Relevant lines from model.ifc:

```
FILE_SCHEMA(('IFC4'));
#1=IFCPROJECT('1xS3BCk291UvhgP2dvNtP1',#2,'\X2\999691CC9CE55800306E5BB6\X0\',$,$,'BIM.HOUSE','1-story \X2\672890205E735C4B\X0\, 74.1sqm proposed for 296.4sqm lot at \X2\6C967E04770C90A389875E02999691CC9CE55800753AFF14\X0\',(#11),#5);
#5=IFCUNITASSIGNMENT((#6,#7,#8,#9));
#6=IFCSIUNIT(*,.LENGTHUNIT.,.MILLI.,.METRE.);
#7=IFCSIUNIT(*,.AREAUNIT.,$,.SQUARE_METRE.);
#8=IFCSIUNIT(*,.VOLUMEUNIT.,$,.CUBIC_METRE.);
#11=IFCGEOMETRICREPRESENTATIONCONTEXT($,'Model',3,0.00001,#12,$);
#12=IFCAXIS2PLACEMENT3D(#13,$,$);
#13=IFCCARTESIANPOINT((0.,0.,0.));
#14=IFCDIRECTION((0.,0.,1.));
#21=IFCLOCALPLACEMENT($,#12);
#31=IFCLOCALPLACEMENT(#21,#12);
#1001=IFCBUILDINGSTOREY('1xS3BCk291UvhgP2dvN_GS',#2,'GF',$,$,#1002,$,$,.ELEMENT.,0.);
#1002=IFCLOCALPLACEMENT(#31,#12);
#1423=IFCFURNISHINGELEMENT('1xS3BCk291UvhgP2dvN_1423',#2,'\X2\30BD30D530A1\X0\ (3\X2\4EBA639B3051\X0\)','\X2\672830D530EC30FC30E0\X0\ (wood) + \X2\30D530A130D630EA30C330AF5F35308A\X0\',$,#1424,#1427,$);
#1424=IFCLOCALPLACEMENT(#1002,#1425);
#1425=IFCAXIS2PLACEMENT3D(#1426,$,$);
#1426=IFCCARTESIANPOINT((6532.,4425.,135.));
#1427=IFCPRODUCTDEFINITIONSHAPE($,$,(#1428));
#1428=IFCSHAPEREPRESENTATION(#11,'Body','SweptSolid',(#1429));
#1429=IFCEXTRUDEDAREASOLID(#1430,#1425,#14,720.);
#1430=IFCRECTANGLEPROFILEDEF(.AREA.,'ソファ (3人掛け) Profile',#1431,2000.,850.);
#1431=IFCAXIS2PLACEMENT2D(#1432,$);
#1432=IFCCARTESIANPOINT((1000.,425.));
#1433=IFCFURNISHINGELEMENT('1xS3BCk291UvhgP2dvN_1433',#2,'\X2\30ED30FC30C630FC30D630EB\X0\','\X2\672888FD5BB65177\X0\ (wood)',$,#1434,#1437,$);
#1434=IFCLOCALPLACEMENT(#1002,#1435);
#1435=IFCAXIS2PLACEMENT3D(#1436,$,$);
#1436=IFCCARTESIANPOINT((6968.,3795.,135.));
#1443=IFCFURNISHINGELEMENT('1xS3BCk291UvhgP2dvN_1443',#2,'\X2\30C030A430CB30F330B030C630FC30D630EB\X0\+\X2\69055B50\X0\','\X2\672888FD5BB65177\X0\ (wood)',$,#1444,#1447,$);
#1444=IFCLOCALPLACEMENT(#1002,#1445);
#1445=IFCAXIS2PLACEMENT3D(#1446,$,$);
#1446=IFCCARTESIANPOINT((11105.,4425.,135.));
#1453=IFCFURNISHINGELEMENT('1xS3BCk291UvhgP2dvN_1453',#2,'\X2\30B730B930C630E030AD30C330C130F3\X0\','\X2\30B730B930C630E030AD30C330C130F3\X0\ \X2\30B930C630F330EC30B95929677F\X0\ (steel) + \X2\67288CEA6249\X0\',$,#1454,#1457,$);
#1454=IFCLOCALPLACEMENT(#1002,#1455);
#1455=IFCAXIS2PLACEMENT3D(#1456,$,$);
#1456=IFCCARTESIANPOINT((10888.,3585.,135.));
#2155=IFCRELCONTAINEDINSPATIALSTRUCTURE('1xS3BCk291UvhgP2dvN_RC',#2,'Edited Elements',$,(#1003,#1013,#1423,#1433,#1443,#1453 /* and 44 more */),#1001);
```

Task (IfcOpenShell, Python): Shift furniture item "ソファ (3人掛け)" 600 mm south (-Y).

```python
import ifcopenshell
import ifcopenshell.api.geometry
import ifcopenshell.util.placement
import ifcopenshell.util.unit

model = ifcopenshell.open("model.ifc")
unit_scale = ifcopenshell.util.unit.calculate_unit_scale(model)

item = model.by_guid("1xS3BCk291UvhgP2dvN_1423")
matrix = ifcopenshell.util.placement.get_local_placement(item.ObjectPlacement)
matrix[1, 3] -= 0.6 / unit_scale
ifcopenshell.api.geometry.edit_object_placement(model, product=item, matrix=matrix, is_si=False)

print(ifcopenshell.util.placement.get_local_placement(item.ObjectPlacement).round(3) + 0.0)

model.write("model_updated.ifc")
```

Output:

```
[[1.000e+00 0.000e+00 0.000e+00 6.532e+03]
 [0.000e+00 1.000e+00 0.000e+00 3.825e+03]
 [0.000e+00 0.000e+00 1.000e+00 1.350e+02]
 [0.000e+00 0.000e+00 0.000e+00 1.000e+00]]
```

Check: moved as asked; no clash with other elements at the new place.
